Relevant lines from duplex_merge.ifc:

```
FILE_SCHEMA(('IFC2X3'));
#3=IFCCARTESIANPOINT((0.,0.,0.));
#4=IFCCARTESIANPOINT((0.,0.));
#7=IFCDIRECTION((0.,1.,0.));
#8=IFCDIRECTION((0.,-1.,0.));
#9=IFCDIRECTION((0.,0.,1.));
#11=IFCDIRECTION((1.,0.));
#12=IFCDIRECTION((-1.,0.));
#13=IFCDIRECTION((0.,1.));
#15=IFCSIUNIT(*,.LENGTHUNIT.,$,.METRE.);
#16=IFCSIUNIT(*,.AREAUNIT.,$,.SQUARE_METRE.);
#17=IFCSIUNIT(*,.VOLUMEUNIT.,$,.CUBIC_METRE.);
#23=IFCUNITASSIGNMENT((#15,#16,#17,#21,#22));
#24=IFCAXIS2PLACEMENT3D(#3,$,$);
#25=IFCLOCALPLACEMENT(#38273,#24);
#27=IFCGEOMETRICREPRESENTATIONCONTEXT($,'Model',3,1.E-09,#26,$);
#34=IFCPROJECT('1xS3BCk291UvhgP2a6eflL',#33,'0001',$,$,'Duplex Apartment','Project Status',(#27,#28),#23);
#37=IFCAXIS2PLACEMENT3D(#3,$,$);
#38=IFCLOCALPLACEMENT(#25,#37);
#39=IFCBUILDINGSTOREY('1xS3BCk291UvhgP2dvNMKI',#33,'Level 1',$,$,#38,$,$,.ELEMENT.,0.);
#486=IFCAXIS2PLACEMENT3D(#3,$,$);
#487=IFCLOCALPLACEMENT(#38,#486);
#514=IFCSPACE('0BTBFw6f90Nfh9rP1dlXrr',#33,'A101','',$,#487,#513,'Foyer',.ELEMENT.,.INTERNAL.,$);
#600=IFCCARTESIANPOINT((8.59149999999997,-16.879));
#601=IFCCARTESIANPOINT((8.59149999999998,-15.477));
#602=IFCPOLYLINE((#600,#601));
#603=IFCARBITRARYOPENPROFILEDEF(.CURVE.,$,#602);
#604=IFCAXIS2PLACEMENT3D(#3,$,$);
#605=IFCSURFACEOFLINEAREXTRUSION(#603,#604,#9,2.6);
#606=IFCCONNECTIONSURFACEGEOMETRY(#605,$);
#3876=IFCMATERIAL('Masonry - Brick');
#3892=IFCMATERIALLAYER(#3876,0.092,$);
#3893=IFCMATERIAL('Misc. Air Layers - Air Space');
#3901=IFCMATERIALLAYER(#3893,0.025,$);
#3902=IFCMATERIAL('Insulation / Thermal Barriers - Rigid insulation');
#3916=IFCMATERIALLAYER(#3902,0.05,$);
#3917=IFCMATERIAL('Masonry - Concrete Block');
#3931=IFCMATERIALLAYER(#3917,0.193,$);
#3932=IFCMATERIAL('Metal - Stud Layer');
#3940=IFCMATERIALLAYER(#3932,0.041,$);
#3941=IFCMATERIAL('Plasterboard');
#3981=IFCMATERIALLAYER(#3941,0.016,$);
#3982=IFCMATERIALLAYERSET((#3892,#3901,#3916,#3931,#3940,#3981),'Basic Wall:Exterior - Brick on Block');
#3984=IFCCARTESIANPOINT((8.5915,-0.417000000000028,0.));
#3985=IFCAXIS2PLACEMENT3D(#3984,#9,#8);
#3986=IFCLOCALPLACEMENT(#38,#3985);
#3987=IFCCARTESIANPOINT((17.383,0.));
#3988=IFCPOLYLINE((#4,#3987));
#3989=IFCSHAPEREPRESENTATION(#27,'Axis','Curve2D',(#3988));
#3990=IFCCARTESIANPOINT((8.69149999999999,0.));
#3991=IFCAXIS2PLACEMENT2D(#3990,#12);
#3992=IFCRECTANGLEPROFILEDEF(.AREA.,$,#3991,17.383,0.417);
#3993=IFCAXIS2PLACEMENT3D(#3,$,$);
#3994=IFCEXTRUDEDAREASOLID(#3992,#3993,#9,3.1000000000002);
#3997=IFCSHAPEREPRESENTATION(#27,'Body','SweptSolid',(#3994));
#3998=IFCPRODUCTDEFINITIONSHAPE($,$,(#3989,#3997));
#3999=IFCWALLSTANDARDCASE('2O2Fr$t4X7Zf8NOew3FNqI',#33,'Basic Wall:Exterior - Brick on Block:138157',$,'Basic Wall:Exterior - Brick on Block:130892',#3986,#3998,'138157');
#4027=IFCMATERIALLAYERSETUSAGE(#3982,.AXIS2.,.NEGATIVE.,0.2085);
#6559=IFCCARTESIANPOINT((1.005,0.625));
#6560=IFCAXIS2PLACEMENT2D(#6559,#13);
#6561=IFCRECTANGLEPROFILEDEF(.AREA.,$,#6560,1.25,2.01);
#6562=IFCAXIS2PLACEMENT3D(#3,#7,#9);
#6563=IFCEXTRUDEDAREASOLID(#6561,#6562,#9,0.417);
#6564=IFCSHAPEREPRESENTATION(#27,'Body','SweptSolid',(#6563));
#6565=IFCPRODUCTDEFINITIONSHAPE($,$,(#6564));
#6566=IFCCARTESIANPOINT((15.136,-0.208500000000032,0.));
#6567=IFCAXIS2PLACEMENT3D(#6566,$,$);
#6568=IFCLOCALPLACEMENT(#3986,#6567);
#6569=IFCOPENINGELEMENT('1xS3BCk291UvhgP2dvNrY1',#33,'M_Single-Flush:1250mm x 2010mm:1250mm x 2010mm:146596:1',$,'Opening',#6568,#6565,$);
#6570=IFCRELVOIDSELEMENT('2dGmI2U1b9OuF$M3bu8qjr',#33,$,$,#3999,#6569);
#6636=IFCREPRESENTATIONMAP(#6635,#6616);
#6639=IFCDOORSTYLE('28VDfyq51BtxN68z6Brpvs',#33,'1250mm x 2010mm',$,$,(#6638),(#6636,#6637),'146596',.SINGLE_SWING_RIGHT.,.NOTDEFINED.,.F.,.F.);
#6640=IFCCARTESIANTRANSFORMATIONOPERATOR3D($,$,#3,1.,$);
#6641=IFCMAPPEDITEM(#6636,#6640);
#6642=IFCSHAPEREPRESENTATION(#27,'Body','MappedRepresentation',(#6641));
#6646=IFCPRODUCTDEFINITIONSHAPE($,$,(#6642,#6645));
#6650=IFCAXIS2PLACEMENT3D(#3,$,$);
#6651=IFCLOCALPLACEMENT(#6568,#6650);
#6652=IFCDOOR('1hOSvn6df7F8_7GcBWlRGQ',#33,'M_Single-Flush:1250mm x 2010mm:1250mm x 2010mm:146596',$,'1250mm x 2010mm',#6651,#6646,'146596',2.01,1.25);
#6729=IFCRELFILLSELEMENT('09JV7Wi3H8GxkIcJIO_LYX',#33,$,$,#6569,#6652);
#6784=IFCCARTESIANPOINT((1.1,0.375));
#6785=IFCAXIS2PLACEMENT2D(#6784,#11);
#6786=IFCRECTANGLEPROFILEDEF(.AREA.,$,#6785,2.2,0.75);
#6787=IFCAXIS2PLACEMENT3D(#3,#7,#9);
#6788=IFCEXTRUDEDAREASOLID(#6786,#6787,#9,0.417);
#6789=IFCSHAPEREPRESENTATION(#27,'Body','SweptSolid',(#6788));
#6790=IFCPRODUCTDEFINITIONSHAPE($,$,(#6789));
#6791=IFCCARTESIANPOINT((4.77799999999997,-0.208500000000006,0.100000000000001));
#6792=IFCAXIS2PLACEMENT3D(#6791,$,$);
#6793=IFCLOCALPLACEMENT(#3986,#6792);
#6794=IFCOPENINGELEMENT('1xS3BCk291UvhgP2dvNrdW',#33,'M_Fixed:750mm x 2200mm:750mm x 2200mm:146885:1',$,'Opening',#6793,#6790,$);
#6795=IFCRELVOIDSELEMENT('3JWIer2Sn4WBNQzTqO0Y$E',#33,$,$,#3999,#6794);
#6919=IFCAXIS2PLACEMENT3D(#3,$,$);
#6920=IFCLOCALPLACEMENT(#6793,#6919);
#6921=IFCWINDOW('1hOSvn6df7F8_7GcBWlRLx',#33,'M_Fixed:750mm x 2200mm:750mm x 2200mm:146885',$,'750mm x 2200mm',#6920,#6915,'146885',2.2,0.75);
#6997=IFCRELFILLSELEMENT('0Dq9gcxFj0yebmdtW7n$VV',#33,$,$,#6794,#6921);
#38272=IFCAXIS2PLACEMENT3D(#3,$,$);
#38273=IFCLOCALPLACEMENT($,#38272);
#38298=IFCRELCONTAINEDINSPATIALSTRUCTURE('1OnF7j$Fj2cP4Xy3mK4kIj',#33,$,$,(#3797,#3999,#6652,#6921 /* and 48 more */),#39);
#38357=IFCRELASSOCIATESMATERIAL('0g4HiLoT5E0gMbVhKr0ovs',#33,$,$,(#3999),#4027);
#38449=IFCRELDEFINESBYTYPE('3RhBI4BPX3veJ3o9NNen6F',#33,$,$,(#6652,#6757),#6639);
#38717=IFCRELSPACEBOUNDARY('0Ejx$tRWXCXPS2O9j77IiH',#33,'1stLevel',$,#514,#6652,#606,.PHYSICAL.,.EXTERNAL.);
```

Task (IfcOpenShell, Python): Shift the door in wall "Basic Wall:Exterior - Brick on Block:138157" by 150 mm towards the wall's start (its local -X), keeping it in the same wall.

```python
import numpy as np
import ifcopenshell
import ifcopenshell.api.geometry
import ifcopenshell.util.placement
import ifcopenshell.util.unit

model = ifcopenshell.open("duplex_merge.ifc")
unit_scale = ifcopenshell.util.unit.calculate_unit_scale(model)

door = model.by_guid("1hOSvn6df7F8_7GcBWlRGQ")
opening = door.FillsVoids[0].RelatingOpeningElement
wall = opening.VoidsElements[0].RelatingBuildingElement

wall_matrix = ifcopenshell.util.placement.get_local_placement(wall.ObjectPlacement)
shift = wall_matrix[:3, 0] * -0.15 / unit_scale
before = ifcopenshell.util.placement.get_local_placement(door.ObjectPlacement)[:3, 3].copy()

# The door is placed relative to its opening, so it follows when the opening moves.
matrix = ifcopenshell.util.placement.get_local_placement(opening.ObjectPlacement)
matrix[:3, 3] += shift
ifcopenshell.api.geometry.edit_object_placement(
    model, product=opening, matrix=matrix, is_si=False, should_transform_children=True
)

# Space boundary surfaces are stored in each space's coordinates; move them too.
for rel in door.ProvidesBoundaries:
    if not rel.ConnectionGeometry:
        continue
    surface = rel.ConnectionGeometry.SurfaceOnRelatingElement
    space_matrix = ifcopenshell.util.placement.get_local_placement(rel.RelatingSpace.ObjectPlacement)
    point = np.array(surface.Position.Location.Coordinates) + space_matrix[:3, :3].T @ shift
    surface.Position = model.createIfcAxis2Placement3D(
        model.createIfcCartesianPoint(point.tolist()), surface.Position.Axis, surface.Position.RefDirection
    )

after = ifcopenshell.util.placement.get_local_placement(door.ObjectPlacement)[:3, 3]
print("door moved by", (after - before).round(3) + 0.0)

model.write("duplex_merge-out.ifc")
```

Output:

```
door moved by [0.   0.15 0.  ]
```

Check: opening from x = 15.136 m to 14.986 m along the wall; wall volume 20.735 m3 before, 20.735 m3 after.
